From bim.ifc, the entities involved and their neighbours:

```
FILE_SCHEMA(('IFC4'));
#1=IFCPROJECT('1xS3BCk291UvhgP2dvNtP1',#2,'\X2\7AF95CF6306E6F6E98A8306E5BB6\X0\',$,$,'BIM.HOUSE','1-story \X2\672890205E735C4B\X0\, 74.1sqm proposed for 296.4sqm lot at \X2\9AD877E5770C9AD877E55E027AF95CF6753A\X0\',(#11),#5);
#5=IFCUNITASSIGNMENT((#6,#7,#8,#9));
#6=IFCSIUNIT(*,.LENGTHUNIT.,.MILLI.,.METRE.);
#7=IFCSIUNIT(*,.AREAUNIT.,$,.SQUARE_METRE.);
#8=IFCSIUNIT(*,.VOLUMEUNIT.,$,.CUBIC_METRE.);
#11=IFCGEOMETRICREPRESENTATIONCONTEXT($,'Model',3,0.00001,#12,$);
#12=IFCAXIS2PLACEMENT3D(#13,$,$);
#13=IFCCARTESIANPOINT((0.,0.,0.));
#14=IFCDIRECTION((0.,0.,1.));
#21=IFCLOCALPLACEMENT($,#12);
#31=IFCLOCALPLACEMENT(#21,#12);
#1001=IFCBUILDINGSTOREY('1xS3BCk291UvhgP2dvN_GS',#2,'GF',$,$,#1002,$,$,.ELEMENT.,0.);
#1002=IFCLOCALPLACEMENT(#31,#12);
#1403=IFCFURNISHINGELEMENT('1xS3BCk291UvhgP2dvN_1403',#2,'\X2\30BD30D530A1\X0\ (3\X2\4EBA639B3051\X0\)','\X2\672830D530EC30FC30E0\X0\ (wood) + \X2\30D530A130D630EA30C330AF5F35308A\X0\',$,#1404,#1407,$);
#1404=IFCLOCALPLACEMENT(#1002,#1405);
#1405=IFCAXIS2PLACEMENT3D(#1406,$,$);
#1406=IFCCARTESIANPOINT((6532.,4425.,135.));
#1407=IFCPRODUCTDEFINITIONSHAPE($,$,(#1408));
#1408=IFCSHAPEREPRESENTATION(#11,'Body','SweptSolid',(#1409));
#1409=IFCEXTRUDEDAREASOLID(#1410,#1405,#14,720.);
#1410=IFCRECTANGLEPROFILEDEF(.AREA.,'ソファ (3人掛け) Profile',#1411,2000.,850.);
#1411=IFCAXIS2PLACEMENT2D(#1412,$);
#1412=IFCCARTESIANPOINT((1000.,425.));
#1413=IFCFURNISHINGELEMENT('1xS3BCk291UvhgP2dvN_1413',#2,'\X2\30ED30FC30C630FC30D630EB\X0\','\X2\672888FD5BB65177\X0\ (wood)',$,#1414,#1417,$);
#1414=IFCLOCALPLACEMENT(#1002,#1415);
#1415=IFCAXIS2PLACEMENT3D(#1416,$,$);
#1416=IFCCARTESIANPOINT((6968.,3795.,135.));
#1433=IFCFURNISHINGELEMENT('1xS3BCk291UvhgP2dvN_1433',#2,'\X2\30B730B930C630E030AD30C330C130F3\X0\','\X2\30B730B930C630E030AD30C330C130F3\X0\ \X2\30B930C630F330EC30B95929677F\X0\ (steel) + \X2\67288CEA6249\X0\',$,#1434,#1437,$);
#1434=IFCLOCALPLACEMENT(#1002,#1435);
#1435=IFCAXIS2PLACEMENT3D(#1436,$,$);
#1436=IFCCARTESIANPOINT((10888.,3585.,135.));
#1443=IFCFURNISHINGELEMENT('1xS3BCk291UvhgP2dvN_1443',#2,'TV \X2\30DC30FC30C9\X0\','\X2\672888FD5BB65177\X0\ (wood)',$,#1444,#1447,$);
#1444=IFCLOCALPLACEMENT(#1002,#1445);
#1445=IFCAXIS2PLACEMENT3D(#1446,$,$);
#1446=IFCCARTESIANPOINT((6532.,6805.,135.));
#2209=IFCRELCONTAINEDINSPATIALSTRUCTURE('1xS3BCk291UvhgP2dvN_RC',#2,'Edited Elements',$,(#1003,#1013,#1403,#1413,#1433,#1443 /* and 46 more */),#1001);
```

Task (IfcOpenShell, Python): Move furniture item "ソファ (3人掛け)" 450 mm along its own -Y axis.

```python
import ifcopenshell
import ifcopenshell.api.geometry
import ifcopenshell.util.placement

model = ifcopenshell.open("bim.ifc")

item = model.by_guid("1xS3BCk291UvhgP2dvN_1403")
matrix = ifcopenshell.util.placement.get_local_placement(item.ObjectPlacement)
matrix[:3, 3] -= matrix[:3, 1] * 450.0
ifcopenshell.api.geometry.edit_object_placement(model, product=item, matrix=matrix, is_si=False)

print(ifcopenshell.util.placement.get_local_placement(item.ObjectPlacement).round(3) + 0.0)

model.write("bim_v2.ifc")
```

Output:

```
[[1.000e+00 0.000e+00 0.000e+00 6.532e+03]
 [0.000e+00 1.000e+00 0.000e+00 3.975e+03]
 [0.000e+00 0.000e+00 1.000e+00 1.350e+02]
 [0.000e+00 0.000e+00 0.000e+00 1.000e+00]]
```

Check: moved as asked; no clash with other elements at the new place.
